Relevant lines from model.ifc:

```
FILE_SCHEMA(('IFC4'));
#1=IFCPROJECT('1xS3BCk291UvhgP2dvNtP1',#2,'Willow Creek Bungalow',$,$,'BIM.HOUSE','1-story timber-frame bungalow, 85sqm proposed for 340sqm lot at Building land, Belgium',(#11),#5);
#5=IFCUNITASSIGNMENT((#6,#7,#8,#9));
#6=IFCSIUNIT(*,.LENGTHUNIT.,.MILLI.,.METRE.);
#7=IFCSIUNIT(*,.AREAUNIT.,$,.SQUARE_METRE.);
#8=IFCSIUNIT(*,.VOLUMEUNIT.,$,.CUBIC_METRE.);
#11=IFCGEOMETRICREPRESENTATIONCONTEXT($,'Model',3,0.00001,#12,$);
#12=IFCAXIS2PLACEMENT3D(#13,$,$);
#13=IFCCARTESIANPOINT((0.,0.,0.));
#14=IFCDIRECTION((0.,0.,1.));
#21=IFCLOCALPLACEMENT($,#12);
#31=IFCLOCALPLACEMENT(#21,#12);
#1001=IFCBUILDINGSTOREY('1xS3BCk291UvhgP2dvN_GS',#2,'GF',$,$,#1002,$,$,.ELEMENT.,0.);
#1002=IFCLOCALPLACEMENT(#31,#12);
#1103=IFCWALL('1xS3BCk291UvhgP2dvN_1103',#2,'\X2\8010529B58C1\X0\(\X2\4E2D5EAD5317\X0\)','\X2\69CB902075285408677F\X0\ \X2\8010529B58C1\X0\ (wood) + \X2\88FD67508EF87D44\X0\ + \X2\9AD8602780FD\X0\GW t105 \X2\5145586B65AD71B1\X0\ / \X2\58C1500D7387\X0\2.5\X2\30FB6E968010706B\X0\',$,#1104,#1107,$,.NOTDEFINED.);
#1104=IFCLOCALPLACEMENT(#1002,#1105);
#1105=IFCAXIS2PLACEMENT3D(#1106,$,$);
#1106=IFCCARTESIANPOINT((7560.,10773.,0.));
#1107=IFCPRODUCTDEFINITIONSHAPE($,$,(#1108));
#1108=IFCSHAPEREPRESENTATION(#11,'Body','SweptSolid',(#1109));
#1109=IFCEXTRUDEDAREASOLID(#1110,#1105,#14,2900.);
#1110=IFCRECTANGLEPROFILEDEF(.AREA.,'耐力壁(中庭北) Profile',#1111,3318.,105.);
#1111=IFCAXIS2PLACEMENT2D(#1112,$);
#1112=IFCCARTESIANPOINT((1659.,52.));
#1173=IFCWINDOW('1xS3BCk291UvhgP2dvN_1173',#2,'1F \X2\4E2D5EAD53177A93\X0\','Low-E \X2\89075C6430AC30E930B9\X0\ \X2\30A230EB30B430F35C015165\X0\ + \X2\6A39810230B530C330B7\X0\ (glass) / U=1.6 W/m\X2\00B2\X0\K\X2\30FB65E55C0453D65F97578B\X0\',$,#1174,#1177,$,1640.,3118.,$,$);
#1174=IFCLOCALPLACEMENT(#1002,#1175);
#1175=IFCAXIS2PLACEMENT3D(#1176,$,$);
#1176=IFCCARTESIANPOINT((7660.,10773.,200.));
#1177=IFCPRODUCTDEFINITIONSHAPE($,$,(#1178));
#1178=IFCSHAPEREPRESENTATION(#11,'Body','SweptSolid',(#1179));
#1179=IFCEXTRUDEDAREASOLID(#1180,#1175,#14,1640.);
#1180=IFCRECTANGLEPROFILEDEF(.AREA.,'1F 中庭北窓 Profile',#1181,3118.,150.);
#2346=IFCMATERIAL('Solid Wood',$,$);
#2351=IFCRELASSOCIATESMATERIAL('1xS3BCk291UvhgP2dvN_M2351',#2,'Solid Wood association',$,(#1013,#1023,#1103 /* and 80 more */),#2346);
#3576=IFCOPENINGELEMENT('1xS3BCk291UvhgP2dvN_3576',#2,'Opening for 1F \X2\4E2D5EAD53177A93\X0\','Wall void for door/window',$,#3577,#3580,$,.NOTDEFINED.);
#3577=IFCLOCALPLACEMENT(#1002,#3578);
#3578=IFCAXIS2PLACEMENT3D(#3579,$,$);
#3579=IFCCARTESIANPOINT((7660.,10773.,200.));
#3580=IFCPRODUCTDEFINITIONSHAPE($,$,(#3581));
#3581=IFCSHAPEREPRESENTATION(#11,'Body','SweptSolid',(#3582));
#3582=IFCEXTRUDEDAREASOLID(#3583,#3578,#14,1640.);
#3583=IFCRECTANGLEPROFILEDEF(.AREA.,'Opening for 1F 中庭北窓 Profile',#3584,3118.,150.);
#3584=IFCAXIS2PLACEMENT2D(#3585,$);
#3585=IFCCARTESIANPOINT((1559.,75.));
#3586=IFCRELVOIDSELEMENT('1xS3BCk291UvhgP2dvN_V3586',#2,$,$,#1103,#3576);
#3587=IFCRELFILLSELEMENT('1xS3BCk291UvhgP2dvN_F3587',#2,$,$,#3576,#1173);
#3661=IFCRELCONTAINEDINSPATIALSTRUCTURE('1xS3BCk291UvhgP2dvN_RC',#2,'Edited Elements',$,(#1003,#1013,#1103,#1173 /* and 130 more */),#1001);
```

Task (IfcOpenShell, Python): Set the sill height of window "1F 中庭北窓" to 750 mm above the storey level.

```python
import numpy as np
import ifcopenshell
import ifcopenshell.api.geometry
import ifcopenshell.geom
import ifcopenshell.util.element
import ifcopenshell.util.placement
import ifcopenshell.util.shape
import ifcopenshell.util.unit

model = ifcopenshell.open("model.ifc")
unit_scale = ifcopenshell.util.unit.calculate_unit_scale(model)

window = model.by_guid("1xS3BCk291UvhgP2dvN_1173")
opening = window.FillsVoids[0].RelatingOpeningElement
storey = ifcopenshell.util.element.get_container(window, ifc_class="IfcBuildingStorey")
level = ifcopenshell.util.placement.get_local_placement(storey.ObjectPlacement)[2, 3]

# The opening's origin need not be at the sill, so measure its lowest point.
shape = ifcopenshell.geom.create_shape(ifcopenshell.geom.settings(), opening)
bottom = ifcopenshell.util.shape.get_shape_bottom_elevation(shape, shape.geometry) / unit_scale
dz = level + 0.75 / unit_scale - bottom

shift = np.array([0.0, 0.0, dz])
# The window is not placed relative to its opening, so move both.
for product in (opening, window):
    matrix = ifcopenshell.util.placement.get_local_placement(product.ObjectPlacement)
    matrix[:3, 3] += shift
    ifcopenshell.api.geometry.edit_object_placement(model, product=product, matrix=matrix, is_si=False)

print(f"moved by {dz * unit_scale:+.3f} m")

model.write("model-out.ifc")
```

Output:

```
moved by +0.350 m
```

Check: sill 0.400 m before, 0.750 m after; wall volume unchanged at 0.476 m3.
